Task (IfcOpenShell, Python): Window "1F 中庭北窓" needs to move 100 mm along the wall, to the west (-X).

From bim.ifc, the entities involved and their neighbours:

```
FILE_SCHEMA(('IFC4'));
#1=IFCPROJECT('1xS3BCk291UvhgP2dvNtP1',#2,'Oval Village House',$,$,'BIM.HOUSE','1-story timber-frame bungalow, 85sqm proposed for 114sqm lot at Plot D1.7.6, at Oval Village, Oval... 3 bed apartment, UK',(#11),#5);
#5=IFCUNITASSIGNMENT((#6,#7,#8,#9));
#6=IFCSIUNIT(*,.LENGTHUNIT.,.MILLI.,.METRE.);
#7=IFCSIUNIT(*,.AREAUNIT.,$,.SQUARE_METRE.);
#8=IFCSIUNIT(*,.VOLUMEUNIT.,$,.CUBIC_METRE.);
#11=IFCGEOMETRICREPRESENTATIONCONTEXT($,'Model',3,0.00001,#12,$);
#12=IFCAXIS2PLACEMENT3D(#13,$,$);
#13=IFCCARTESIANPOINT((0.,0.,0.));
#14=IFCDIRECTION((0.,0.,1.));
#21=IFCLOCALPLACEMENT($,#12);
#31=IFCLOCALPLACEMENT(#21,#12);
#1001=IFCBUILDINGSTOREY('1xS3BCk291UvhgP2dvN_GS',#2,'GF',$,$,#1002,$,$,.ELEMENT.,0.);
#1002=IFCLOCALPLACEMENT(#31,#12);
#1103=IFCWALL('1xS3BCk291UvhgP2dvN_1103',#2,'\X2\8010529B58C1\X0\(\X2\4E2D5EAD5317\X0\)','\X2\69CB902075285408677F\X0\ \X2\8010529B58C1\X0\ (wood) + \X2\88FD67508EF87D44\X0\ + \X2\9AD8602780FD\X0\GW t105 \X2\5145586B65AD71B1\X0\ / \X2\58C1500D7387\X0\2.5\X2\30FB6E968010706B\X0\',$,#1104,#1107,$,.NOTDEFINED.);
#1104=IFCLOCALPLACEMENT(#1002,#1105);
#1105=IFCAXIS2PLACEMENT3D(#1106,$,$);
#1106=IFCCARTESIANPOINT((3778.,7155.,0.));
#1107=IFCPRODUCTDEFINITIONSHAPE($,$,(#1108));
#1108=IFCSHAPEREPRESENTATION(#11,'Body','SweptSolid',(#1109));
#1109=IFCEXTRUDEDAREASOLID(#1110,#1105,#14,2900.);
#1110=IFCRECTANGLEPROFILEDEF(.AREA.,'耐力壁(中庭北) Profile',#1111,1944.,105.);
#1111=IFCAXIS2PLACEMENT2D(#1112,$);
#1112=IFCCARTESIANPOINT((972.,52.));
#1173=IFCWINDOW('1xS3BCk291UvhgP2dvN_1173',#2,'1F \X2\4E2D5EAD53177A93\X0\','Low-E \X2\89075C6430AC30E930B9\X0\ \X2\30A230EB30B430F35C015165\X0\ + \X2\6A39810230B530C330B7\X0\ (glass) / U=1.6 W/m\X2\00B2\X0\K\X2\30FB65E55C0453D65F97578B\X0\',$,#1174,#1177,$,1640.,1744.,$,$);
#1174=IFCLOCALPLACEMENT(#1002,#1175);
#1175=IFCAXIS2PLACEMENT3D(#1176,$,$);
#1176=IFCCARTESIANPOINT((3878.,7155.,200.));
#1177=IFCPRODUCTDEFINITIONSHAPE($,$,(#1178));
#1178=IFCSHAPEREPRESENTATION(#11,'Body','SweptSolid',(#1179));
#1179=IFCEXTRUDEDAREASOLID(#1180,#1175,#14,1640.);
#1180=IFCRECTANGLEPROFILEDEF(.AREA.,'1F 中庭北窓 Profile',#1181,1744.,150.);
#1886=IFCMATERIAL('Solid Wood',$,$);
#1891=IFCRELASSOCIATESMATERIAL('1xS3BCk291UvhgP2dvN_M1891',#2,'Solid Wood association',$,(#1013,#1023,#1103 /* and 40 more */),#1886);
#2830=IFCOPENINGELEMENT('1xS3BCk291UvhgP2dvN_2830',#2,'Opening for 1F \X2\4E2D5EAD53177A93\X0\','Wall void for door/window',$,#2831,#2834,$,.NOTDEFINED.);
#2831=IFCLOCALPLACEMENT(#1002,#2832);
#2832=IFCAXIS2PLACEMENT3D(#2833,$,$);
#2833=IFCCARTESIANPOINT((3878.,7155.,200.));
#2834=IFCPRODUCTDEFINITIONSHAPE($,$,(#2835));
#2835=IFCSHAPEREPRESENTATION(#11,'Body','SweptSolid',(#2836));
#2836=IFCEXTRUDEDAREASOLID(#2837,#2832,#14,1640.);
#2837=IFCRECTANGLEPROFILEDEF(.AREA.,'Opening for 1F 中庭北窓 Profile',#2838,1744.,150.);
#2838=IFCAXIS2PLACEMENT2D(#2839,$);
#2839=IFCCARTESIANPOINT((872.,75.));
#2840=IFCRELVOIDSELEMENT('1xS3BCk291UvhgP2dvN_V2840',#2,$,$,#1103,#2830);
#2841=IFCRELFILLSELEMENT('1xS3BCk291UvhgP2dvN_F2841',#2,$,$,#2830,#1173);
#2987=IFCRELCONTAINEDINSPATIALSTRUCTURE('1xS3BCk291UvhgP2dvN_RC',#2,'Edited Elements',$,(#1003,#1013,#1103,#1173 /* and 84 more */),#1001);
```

```python
import ifcopenshell
import ifcopenshell.api.geometry
import ifcopenshell.util.placement

model = ifcopenshell.open("bim.ifc")

window = model.by_guid("1xS3BCk291UvhgP2dvN_1173")
opening = window.FillsVoids[0].RelatingOpeningElement
wall = opening.VoidsElements[0].RelatingBuildingElement

wall_matrix = ifcopenshell.util.placement.get_local_placement(wall.ObjectPlacement)
shift = wall_matrix[:3, 0] * -100.0
before = ifcopenshell.util.placement.get_local_placement(window.ObjectPlacement)[:3, 3].copy()

# The window is not placed relative to its opening, so move both.
for product in (opening, window):
    matrix = ifcopenshell.util.placement.get_local_placement(product.ObjectPlacement)
    matrix[:3, 3] += shift
    ifcopenshell.api.geometry.edit_object_placement(model, product=product, matrix=matrix, is_si=False)

after = ifcopenshell.util.placement.get_local_placement(window.ObjectPlacement)[:3, 3]
print("window moved by", (after - before).round(3) + 0.0)

model.write("bim_v2.ifc")
```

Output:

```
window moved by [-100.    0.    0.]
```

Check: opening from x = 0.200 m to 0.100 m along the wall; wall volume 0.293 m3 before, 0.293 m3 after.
